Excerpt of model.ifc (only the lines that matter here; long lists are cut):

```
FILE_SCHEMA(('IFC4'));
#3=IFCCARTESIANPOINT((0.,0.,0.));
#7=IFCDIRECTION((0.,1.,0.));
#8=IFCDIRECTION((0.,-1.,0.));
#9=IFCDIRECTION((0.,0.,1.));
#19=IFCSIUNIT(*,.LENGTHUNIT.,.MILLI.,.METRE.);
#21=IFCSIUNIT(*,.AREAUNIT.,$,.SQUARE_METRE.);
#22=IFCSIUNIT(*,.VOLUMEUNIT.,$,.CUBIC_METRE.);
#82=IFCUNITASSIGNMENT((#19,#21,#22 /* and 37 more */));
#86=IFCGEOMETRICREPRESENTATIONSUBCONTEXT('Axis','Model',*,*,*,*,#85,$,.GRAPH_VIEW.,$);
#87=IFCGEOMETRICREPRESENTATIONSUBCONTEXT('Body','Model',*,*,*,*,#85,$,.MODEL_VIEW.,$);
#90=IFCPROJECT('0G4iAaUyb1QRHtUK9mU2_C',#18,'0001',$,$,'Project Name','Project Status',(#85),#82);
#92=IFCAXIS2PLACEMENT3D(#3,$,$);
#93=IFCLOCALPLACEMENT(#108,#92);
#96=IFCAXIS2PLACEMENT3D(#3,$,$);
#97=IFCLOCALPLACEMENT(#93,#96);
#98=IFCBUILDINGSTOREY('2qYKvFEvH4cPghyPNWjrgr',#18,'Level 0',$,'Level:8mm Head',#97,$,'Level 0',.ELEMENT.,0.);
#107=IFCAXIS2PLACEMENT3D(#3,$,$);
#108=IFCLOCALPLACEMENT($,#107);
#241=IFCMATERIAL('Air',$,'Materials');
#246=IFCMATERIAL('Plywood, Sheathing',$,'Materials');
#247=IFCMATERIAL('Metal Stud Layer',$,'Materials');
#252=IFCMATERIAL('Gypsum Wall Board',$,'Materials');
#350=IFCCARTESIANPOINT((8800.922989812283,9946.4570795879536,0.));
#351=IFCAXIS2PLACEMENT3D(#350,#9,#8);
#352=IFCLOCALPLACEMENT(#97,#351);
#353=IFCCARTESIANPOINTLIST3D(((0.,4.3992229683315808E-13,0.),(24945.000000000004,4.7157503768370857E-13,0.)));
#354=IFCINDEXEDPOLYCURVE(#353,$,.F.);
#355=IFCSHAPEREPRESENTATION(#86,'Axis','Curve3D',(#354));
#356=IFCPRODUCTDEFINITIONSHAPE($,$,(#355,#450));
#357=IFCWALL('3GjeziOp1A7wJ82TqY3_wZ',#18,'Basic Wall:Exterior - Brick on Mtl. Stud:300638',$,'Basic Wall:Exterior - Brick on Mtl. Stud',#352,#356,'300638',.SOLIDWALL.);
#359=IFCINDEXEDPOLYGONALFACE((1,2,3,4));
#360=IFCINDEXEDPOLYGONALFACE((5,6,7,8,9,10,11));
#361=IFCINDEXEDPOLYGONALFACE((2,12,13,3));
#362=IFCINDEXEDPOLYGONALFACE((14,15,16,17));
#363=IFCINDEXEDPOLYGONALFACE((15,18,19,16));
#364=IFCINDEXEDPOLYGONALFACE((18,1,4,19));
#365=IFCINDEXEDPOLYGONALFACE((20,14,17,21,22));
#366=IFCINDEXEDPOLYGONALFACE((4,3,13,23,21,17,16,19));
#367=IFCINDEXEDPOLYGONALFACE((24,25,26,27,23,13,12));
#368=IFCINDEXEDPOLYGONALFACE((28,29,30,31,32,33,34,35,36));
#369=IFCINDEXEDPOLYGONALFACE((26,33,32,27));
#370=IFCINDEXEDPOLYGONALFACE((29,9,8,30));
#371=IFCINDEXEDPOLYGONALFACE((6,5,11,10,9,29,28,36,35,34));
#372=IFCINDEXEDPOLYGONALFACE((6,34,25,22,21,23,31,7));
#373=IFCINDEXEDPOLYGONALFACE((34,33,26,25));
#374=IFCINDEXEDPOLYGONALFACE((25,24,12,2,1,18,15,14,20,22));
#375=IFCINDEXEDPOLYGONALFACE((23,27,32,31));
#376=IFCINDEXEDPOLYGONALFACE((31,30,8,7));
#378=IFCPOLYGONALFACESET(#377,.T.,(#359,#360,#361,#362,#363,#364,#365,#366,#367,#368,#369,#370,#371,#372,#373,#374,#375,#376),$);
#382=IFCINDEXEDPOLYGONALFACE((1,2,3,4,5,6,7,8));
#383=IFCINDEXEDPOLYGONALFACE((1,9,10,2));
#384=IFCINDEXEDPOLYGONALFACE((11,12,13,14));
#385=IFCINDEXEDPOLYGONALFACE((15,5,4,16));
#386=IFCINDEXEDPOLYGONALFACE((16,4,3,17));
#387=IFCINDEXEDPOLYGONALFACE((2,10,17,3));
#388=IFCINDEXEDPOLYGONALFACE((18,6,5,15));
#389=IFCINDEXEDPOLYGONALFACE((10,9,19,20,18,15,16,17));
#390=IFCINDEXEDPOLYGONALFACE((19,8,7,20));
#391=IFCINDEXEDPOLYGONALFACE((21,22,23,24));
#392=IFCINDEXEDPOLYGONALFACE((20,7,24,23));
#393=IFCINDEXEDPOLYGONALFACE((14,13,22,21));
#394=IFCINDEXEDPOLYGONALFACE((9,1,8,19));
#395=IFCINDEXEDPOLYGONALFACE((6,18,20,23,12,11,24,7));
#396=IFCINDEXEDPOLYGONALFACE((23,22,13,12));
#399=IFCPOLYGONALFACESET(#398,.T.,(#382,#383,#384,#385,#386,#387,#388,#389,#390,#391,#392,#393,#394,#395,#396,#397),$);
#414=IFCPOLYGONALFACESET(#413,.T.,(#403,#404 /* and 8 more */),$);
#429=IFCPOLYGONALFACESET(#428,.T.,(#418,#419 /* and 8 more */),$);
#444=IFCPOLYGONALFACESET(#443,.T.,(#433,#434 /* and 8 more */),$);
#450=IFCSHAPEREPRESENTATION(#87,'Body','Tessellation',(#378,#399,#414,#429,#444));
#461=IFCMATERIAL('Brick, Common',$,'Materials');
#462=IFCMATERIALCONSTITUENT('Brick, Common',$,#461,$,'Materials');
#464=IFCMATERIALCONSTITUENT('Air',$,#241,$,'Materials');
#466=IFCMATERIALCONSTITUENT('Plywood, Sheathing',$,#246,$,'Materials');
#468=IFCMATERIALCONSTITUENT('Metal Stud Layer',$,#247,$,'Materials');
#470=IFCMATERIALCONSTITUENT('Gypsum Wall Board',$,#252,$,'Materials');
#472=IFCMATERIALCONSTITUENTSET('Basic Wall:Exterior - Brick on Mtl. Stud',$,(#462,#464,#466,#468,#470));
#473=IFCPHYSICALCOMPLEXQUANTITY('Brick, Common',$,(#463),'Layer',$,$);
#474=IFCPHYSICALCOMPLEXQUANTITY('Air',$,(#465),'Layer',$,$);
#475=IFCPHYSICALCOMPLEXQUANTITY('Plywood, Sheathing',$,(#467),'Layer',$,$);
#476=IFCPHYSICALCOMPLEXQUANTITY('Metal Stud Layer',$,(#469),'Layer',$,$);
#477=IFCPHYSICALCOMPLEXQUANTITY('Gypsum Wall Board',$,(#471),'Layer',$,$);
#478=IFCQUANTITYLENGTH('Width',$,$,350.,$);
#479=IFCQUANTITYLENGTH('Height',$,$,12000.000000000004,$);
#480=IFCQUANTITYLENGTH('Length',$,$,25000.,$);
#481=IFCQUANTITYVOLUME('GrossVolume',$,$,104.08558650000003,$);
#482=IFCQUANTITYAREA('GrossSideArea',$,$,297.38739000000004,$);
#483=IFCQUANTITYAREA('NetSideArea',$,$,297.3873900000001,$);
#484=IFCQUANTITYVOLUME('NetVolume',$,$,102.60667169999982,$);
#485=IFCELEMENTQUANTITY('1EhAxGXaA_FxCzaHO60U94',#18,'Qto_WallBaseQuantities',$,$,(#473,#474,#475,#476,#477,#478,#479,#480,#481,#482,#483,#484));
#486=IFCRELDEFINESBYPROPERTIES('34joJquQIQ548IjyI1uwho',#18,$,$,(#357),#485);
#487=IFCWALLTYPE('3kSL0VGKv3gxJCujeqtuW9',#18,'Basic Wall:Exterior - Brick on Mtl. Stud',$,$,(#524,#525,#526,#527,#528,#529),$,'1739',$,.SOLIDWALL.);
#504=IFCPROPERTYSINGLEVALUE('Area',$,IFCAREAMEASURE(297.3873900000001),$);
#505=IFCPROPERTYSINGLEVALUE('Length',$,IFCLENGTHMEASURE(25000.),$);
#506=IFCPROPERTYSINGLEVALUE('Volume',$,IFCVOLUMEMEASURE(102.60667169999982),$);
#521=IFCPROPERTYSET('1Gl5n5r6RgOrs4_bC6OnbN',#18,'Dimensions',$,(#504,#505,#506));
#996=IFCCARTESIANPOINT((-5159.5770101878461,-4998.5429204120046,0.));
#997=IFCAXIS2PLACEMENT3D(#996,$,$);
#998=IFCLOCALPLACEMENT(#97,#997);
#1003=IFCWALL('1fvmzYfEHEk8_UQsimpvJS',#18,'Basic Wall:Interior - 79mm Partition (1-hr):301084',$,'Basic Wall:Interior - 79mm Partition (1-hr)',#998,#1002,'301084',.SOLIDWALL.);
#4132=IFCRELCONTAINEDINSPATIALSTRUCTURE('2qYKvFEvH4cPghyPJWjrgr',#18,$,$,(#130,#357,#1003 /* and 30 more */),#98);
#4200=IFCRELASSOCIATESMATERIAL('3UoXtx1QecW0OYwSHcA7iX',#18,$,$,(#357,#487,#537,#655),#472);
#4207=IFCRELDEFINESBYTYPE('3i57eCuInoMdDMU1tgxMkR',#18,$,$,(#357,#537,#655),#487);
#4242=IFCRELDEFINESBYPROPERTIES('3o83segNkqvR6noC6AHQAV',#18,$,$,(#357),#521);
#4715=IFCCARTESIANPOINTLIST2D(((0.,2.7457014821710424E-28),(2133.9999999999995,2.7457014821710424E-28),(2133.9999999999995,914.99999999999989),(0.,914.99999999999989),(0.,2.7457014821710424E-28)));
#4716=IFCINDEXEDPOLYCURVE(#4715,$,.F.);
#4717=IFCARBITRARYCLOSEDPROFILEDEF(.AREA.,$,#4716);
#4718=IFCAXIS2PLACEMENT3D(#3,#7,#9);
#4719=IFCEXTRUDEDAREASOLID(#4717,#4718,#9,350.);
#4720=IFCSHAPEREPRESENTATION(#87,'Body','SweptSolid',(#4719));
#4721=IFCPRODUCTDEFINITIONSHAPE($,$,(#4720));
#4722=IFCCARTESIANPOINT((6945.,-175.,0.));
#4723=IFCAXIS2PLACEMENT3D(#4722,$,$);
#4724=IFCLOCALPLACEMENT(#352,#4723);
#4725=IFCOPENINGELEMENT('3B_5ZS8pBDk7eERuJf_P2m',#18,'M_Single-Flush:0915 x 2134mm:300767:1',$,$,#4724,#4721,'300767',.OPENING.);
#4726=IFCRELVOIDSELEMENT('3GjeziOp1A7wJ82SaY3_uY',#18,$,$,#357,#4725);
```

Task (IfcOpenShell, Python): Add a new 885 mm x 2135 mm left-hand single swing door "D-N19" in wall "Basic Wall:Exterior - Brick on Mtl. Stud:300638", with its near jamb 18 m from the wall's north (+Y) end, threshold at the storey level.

```python
import numpy as np
import ifcopenshell
import ifcopenshell.api.feature
import ifcopenshell.api.geometry
import ifcopenshell.api.pset
import ifcopenshell.api.root
import ifcopenshell.api.spatial
import ifcopenshell.geom
import ifcopenshell.util.element
import ifcopenshell.util.placement
import ifcopenshell.util.representation
import ifcopenshell.util.shape
import ifcopenshell.util.unit

model = ifcopenshell.open("model.ifc")
unit_scale = ifcopenshell.util.unit.calculate_unit_scale(model)
area_scale = ifcopenshell.util.unit.calculate_unit_scale(model, "AREAUNIT")
volume_scale = ifcopenshell.util.unit.calculate_unit_scale(model, "VOLUMEUNIT")
settings = ifcopenshell.geom.settings()


def volume(element):
    """Net volume in cubic metres, openings subtracted."""
    shape = ifcopenshell.geom.create_shape(settings, element)
    return ifcopenshell.util.shape.get_volume(shape.geometry)


wall = model.by_guid("3GjeziOp1A7wJ82TqY3_wZ")
storey = ifcopenshell.util.element.get_container(wall, ifc_class="IfcBuildingStorey")
context = ifcopenshell.util.representation.get_context(model, "Model", "Body", "MODEL_VIEW")
before = volume(wall)

width, height, from_end, sill = 0.885, 2.135, 18, 0.0  # metres

# The wall runs along its own X axis, and the end named is its -X end.
wall_shape = ifcopenshell.geom.create_shape(settings, wall)
x, y, z = ifcopenshell.util.shape.get_vertices(wall_shape.geometry).T
start = x.min() + from_end
face, thickness = float(y.min()), float(y.max() - y.min())
wall_matrix = ifcopenshell.util.placement.get_local_placement(wall.ObjectPlacement)
level = ifcopenshell.util.placement.get_local_placement(storey.ObjectPlacement)[2, 3]


def in_wall(x, y):
    """Placement at x, y metres in the wall's axes, at sill height."""
    matrix = wall_matrix.copy()
    matrix[:, 3] = wall_matrix @ np.array([x / unit_scale, y / unit_scale, 0.0, 1.0])
    matrix[2, 3] = level + sill / unit_scale
    return matrix


# Opening: a box that overshoots both wall faces by 50 mm.
opening = ifcopenshell.api.root.create_entity(model, ifc_class="IfcOpeningElement", predefined_type="OPENING")
box = ifcopenshell.api.geometry.add_wall_representation(
    model, context=context, length=width, height=height, thickness=thickness + 0.1
)
ifcopenshell.api.geometry.assign_representation(model, product=opening, representation=box)
ifcopenshell.api.geometry.edit_object_placement(model, product=opening, matrix=in_wall(start, face - 0.05), is_si=False)
ifcopenshell.api.feature.add_feature(model, feature=opening, element=wall)

door = ifcopenshell.api.root.create_entity(model, ifc_class="IfcDoor", name="D-N19", predefined_type="DOOR")
door.OverallWidth, door.OverallHeight = width / unit_scale, height / unit_scale
door.OperationType = "SINGLE_SWING_LEFT"
body = ifcopenshell.api.geometry.add_door_representation(
    model,
    context=context,
    overall_width=door.OverallWidth,
    overall_height=door.OverallHeight,
    operation_type="SINGLE_SWING_LEFT",
    lining_properties={"LiningDepth": thickness / unit_scale, "ThresholdDepth": thickness / unit_scale},
)
ifcopenshell.api.geometry.assign_representation(model, product=door, representation=body)
ifcopenshell.api.spatial.assign_container(model, products=[door], relating_structure=storey)
ifcopenshell.api.feature.add_filling(model, opening=opening, element=door)

# The lining spans the wall, so the door starts at the wall face.
ifcopenshell.api.geometry.edit_object_placement(model, product=door, matrix=in_wall(start, face), is_si=False)

after = volume(wall)

# Update the wall's stored quantities.
qto = model.by_id(ifcopenshell.util.element.get_pset(wall, "Qto_WallBaseQuantities", should_inherit=False)["id"])
ifcopenshell.api.pset.edit_qto(model, qto=qto, properties={
    "NetSideArea": after / thickness / area_scale,
    "NetVolume": after / volume_scale,
})
pset = model.by_id(ifcopenshell.util.element.get_pset(wall, "Dimensions", should_inherit=False)["id"])
ifcopenshell.api.pset.edit_pset(model, pset=pset, properties={
    "Area": model.create_entity("IfcAreaMeasure", after / thickness / area_scale),
    "Volume": model.create_entity("IfcVolumeMeasure", after / volume_scale),
})

print(f"wall volume {before:.3f} -> {after:.3f} m3")

model.write("model-out.ifc")
```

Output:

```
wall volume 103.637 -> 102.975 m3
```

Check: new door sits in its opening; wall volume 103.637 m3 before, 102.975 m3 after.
